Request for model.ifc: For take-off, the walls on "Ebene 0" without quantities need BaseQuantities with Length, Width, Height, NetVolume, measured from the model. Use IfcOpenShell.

First a look at what the model holds.

```python
import ifcopenshell
import ifcopenshell.util.element
import ifcopenshell.util.unit

model = ifcopenshell.open("model.ifc")
print(model.schema)
for unit_type in ("LENGTHUNIT", "AREAUNIT", "VOLUMEUNIT"):
    print(unit_type, ifcopenshell.util.unit.calculate_unit_scale(model, unit_type))
storey = next(s for s in model.by_type("IfcBuildingStorey") if s.Name == "Ebene 0")
walls = [e for e in ifcopenshell.util.element.get_decomposition(storey) if e.is_a("IfcWall")]
for e in sorted(walls, key=lambda e: e.id()):
    print(e.id(), e.is_a(), e.Name, list(ifcopenshell.util.element.get_psets(e, qtos_only=True)), sep=" | ")
```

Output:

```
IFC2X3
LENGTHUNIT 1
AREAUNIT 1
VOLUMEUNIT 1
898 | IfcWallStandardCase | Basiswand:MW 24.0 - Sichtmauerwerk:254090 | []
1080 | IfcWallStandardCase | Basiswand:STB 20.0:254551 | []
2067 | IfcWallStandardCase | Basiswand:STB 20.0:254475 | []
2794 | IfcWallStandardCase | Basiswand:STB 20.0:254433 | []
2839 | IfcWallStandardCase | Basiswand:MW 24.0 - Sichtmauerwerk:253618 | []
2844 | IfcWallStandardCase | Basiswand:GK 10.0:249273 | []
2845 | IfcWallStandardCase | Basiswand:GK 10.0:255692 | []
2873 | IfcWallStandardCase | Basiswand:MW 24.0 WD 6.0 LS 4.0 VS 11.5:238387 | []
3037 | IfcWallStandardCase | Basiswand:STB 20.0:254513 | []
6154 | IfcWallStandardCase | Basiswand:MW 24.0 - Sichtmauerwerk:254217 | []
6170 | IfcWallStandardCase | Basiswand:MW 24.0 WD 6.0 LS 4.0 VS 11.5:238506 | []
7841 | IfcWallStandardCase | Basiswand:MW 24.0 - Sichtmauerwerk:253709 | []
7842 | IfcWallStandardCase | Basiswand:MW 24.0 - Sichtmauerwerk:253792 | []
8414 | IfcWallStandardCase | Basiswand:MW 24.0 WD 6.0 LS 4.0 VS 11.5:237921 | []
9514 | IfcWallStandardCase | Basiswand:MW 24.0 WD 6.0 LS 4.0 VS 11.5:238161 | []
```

```python
import ifcopenshell
import ifcopenshell.api.pset
import ifcopenshell.geom
import ifcopenshell.util.element
import ifcopenshell.util.shape
import ifcopenshell.util.unit

model = ifcopenshell.open("model.ifc")
unit_scale = ifcopenshell.util.unit.calculate_unit_scale(model)
volume_scale = ifcopenshell.util.unit.calculate_unit_scale(model, "VOLUMEUNIT")
settings = ifcopenshell.geom.settings()

storey = next(s for s in model.by_type("IfcBuildingStorey") if s.Name == "Ebene 0")
walls = [e for e in ifcopenshell.util.element.get_decomposition(storey) if e.is_a("IfcWall")]

for e in sorted(walls, key=lambda e: e.id()):
    if ifcopenshell.util.element.get_psets(e, qtos_only=True, should_inherit=False):
        continue
    # Geometry comes back in metres, in the element's own axes.
    shape = ifcopenshell.geom.create_shape(settings, e)
    values = {
        "Length": ifcopenshell.util.shape.get_x(shape.geometry) / unit_scale,
        "Width": ifcopenshell.util.shape.get_y(shape.geometry) / unit_scale,
        "Height": ifcopenshell.util.shape.get_z(shape.geometry) / unit_scale,
        "NetVolume": ifcopenshell.util.shape.get_volume(shape.geometry) / volume_scale,
    }
    qto = ifcopenshell.api.pset.add_qto(model, product=e, name="BaseQuantities")
    ifcopenshell.api.pset.edit_qto(model, qto=qto, properties=values)
    print(e.id(), {k: round(v, 3) for k, v in values.items()})

model.write("model_rev.ifc")
```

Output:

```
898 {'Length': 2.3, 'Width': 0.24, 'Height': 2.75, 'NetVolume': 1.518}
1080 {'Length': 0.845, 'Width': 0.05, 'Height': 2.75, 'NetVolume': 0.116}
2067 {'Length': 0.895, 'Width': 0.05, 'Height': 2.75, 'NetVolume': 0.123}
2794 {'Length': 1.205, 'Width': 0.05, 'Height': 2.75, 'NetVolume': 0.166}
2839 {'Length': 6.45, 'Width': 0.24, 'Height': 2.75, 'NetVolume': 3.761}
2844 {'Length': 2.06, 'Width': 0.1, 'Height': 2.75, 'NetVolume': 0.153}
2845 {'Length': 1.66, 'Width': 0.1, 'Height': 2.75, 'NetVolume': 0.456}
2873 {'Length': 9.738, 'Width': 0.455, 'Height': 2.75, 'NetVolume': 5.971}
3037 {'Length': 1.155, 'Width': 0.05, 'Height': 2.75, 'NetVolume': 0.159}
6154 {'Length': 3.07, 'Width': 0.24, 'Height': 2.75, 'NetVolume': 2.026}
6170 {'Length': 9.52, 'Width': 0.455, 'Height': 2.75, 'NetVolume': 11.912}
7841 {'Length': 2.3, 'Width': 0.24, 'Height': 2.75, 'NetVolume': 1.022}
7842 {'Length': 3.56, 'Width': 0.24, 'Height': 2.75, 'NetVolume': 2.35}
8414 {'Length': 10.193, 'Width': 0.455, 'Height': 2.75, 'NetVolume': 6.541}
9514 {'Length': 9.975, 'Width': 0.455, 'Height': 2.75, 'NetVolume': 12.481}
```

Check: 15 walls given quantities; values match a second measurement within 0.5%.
